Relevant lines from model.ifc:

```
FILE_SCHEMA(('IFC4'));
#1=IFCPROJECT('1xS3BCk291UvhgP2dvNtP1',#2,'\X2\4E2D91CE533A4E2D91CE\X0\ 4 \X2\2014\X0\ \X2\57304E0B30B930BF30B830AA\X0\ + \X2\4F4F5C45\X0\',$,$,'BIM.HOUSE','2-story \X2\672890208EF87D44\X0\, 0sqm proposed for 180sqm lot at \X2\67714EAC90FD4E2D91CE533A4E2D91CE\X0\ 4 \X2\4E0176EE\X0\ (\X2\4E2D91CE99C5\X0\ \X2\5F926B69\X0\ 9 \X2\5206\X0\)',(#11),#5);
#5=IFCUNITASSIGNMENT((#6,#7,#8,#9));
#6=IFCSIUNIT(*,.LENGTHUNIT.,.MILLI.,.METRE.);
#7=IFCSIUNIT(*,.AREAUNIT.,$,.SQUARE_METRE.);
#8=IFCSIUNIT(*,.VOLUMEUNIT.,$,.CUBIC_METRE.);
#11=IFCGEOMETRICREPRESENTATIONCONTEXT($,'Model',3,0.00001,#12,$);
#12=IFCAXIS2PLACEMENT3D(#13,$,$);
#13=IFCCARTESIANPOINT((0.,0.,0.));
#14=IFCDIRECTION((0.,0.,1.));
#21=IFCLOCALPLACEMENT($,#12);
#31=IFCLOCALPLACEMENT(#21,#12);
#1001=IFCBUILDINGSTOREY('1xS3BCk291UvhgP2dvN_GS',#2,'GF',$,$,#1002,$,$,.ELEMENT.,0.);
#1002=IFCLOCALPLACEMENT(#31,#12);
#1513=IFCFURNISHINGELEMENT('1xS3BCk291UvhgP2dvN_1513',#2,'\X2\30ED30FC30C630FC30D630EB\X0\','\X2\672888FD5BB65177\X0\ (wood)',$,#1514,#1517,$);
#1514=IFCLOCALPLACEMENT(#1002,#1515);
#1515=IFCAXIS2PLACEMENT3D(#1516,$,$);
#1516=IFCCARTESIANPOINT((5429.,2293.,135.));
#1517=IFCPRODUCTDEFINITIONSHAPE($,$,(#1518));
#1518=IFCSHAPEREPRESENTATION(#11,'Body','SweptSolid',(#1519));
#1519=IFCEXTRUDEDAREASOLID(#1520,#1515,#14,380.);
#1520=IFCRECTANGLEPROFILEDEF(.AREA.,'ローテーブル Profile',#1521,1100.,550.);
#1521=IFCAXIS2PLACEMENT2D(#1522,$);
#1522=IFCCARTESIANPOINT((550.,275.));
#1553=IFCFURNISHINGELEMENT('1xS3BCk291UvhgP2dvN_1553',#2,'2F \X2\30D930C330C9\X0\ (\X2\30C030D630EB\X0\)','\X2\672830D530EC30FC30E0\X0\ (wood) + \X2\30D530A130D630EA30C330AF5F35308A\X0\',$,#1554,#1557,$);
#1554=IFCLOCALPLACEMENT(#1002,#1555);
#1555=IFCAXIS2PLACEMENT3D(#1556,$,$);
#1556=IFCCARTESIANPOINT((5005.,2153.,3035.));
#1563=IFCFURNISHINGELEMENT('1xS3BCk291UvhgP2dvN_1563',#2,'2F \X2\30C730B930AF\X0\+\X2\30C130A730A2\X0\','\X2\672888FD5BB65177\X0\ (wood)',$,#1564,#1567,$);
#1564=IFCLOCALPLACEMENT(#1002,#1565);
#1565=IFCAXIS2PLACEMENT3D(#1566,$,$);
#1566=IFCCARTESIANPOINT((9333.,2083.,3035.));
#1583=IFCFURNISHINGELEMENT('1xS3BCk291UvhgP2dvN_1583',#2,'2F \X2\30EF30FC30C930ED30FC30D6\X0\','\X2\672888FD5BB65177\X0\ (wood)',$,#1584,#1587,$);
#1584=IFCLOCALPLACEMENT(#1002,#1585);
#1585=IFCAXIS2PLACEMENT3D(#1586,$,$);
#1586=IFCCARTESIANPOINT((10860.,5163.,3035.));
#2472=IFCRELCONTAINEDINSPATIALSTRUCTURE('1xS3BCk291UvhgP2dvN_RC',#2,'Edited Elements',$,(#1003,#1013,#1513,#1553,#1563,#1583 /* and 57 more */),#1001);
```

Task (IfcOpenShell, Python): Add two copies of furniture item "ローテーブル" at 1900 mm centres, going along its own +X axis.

```python
import ifcopenshell
import ifcopenshell.api.geometry
import ifcopenshell.api.root
import ifcopenshell.util.element
import ifcopenshell.util.placement
import ifcopenshell.util.unit

model = ifcopenshell.open("model.ifc")
unit_scale = ifcopenshell.util.unit.calculate_unit_scale(model)


def reuse_history(source, copy):
    """copy_class also copies each property set's owner history, people and application; keep the originals."""
    for rel in copy.IsDefinedBy:
        if rel.is_a("IfcRelDefinesByProperties") and (history := rel.RelatingPropertyDefinition.OwnerHistory):
            rel.RelatingPropertyDefinition.OwnerHistory = source.OwnerHistory
            ifcopenshell.util.element.remove_deep2(model, history)


source = model.by_id(1513)
base = ifcopenshell.util.placement.get_local_placement(source.ObjectPlacement)
step = base[:3, 0] * 1.9 / unit_scale

for i in range(1, 3):
    copy = ifcopenshell.api.root.copy_class(model, product=source)
    copy.Representation = ifcopenshell.util.element.copy_deep(
        model, source.Representation, exclude=["IfcGeometricRepresentationContext", "IfcRepresentationMap"]
    )
    reuse_history(source, copy)
    matrix = base.copy()
    matrix[:3, 3] += i * step
    print("added at", matrix[:3, 3].round(3) + 0.0)
    ifcopenshell.api.geometry.edit_object_placement(model, product=copy, matrix=matrix, is_si=False)

model.write("model_updated.ifc")
```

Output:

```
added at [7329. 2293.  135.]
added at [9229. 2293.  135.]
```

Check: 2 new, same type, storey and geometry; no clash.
